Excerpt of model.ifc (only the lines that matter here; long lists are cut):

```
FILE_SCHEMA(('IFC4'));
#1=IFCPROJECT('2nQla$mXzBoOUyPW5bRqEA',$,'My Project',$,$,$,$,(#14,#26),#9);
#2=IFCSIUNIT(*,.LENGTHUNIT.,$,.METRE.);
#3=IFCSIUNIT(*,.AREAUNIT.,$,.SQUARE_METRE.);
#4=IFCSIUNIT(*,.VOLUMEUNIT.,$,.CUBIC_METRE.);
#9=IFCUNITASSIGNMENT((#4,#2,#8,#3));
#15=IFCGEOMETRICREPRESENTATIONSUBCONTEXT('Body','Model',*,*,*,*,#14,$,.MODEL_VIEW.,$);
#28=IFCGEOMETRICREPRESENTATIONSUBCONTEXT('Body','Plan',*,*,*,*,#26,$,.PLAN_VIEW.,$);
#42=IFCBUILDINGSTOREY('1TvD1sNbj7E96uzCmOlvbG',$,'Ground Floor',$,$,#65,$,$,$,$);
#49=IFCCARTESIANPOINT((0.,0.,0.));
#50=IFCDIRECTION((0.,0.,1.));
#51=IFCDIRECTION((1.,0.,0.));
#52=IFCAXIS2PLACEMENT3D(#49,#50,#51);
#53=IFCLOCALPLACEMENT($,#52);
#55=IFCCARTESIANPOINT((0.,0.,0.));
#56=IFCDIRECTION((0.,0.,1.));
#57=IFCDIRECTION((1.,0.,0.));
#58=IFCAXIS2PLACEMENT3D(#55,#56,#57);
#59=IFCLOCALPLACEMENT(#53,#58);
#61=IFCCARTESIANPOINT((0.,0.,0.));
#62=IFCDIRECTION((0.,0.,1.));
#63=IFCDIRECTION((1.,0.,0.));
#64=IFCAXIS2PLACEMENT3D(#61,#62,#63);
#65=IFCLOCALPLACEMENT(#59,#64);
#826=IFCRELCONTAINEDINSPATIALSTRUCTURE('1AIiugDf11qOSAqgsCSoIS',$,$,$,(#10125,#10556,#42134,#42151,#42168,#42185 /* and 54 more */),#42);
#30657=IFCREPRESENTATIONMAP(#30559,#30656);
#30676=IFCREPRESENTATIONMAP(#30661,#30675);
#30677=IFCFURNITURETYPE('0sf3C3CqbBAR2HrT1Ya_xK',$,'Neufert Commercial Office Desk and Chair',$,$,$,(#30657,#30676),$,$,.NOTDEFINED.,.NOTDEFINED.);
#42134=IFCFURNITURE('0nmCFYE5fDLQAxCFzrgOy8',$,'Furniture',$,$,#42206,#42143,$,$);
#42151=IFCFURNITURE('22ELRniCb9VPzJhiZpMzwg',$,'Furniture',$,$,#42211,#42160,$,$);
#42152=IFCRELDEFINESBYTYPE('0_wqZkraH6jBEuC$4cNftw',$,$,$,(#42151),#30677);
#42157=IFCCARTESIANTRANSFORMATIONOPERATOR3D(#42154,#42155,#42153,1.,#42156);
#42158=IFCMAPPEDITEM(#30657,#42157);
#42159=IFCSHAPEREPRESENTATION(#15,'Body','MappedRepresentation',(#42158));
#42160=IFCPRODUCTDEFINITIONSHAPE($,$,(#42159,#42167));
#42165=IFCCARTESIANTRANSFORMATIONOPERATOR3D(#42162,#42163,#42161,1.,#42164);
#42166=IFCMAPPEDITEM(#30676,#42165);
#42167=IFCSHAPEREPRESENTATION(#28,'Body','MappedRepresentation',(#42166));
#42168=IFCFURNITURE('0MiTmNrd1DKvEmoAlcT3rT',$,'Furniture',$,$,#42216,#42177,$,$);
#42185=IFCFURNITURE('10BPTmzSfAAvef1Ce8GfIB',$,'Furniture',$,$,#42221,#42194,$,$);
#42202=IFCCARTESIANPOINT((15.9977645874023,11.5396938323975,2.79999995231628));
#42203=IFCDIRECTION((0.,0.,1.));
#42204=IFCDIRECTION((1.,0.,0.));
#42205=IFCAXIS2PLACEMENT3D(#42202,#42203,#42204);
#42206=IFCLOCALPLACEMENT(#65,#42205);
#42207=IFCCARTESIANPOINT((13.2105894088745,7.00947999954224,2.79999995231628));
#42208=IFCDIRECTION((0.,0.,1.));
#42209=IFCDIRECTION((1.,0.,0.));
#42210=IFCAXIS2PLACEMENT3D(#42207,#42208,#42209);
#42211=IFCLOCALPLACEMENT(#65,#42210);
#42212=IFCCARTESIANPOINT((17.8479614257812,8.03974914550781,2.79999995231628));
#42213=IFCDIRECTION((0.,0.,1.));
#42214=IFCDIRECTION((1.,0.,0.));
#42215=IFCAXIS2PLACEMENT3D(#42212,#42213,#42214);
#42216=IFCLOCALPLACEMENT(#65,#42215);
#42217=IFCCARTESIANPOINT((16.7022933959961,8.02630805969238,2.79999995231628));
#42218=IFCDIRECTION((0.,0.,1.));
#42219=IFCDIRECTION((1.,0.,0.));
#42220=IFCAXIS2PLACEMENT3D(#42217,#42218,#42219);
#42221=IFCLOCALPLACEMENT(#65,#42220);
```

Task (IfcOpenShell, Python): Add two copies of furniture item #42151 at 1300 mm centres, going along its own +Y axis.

```python
import ifcopenshell
import ifcopenshell.api.geometry
import ifcopenshell.api.root
import ifcopenshell.util.element
import ifcopenshell.util.placement
import ifcopenshell.util.unit

model = ifcopenshell.open("model.ifc")
unit_scale = ifcopenshell.util.unit.calculate_unit_scale(model)

source = model.by_guid("22ELRniCb9VPzJhiZpMzwg")
base = ifcopenshell.util.placement.get_local_placement(source.ObjectPlacement)
step = base[:3, 1] * 1.3 / unit_scale

for i in range(1, 3):
    copy = ifcopenshell.api.root.copy_class(model, product=source)
    copy.Representation = ifcopenshell.util.element.copy_deep(
        model, source.Representation, exclude=["IfcGeometricRepresentationContext", "IfcRepresentationMap"]
    )
    matrix = base.copy()
    matrix[:3, 3] += i * step
    print("added at", matrix[:3, 3].round(3) + 0.0)
    ifcopenshell.api.geometry.edit_object_placement(model, product=copy, matrix=matrix, is_si=False)

model.write("model_rev.ifc")
```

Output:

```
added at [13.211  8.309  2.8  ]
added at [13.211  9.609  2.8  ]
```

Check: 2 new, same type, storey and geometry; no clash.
